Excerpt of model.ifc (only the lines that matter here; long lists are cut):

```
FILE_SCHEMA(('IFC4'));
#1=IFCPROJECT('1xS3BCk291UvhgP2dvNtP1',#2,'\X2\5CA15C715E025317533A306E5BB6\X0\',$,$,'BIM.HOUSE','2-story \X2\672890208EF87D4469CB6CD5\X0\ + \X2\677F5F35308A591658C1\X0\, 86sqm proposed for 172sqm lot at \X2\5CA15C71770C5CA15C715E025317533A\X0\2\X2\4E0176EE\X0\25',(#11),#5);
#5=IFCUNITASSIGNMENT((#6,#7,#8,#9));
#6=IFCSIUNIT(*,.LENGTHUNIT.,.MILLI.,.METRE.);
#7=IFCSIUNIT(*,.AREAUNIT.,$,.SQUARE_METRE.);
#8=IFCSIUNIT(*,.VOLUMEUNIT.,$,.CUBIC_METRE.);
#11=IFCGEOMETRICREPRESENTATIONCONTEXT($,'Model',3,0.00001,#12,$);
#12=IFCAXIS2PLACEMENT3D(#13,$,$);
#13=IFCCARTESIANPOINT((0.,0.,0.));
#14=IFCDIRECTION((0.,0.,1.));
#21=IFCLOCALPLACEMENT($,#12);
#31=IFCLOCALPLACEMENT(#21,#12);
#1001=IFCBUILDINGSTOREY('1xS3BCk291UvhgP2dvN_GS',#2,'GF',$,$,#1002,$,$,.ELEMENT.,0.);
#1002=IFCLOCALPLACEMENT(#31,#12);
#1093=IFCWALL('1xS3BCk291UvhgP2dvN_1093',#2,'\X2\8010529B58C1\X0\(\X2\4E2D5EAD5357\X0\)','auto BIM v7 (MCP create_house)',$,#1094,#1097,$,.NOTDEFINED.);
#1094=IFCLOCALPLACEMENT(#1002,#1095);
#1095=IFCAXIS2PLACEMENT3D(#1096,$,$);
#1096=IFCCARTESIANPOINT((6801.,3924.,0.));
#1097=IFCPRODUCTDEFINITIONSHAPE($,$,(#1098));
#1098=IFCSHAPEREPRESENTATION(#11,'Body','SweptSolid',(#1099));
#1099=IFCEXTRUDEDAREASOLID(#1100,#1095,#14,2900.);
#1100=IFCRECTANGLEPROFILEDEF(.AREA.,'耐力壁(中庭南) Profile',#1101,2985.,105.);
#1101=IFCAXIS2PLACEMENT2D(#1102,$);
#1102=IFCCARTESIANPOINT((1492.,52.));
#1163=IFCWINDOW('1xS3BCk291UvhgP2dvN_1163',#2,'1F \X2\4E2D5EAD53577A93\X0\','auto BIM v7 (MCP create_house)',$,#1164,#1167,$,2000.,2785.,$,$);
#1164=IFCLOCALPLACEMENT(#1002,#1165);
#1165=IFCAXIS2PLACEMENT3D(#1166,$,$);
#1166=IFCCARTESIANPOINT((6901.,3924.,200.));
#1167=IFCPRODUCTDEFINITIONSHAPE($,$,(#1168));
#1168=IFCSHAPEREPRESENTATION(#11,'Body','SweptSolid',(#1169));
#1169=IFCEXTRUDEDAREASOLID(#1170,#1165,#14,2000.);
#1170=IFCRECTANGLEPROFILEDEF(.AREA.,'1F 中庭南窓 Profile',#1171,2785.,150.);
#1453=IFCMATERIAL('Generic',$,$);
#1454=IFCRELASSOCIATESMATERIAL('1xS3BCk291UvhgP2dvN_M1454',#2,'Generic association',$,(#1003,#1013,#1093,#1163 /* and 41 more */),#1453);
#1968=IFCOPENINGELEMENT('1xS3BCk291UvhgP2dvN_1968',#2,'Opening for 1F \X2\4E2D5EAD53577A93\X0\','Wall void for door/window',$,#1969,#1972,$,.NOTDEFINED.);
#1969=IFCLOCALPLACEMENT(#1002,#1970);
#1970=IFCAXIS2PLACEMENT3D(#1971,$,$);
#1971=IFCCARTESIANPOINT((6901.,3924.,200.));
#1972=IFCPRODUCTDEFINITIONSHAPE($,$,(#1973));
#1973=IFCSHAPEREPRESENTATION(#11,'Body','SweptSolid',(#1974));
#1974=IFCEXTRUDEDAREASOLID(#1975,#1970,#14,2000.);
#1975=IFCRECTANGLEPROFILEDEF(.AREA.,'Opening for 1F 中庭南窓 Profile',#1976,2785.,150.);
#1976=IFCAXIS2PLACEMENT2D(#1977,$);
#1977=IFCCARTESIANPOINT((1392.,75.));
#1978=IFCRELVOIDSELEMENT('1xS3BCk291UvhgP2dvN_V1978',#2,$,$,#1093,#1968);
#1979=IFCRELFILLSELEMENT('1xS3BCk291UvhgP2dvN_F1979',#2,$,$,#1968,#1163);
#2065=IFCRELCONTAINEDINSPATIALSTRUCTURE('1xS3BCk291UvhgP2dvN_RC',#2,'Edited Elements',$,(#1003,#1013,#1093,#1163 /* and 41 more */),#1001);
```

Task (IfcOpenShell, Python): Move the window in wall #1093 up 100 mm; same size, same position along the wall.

```python
import numpy as np
import ifcopenshell
import ifcopenshell.api.geometry
import ifcopenshell.util.placement
import ifcopenshell.util.unit

model = ifcopenshell.open("model.ifc")
unit_scale = ifcopenshell.util.unit.calculate_unit_scale(model)

window = model.by_id(1163)
opening = window.FillsVoids[0].RelatingOpeningElement
dz = 100.0

shift = np.array([0.0, 0.0, dz])
# The window is not placed relative to its opening, so move both.
for product in (opening, window):
    matrix = ifcopenshell.util.placement.get_local_placement(product.ObjectPlacement)
    matrix[:3, 3] += shift
    ifcopenshell.api.geometry.edit_object_placement(model, product=product, matrix=matrix, is_si=False)

print(f"moved by {dz * unit_scale:+.3f} m")

model.write("model_edited.ifc")
```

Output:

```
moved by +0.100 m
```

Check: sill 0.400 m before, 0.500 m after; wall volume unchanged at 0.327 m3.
